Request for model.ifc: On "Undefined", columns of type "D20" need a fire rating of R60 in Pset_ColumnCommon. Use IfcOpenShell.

First a look at what the model holds.

```python
import ifcopenshell
import ifcopenshell.util.element

model = ifcopenshell.open("model.ifc")
print(model.schema)
storey = next(s for s in model.by_type("IfcBuildingStorey") if s.Name == "Undefined")
columns = [e for e in ifcopenshell.util.element.get_decomposition(storey) if e.is_a("IfcColumn")]
seen = {}
for e in columns:
    element_type = ifcopenshell.util.element.get_type(e)
    key = (element_type.Name if element_type != e and element_type else None, ifcopenshell.util.element.get_pset(e, "Pset_ColumnCommon", "FireRating"))
    seen[key] = seen.get(key, 0) + 1
for (name, value), count in sorted(seen.items(), key=str):
    print(count, "x", name, "|", value)
```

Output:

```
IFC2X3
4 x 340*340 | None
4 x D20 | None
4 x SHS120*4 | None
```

```python
import ifcopenshell
import ifcopenshell.api.pset
import ifcopenshell.util.element

model = ifcopenshell.open("model.ifc")

storey = next(s for s in model.by_type("IfcBuildingStorey") if s.Name == "Undefined")
columns = [e for e in ifcopenshell.util.element.get_decomposition(storey) if e.is_a("IfcColumn")]

count = 0
for e in columns:
    element_type = ifcopenshell.util.element.get_type(e)
    if element_type in (None, e) or element_type.Name != "D20":
        continue
    # add_pset returns the element's existing set when there is one.
    pset = ifcopenshell.api.pset.add_pset(model, product=e, name="Pset_ColumnCommon")
    ifcopenshell.api.pset.edit_pset(model, pset=pset, properties={"FireRating": "R60"})
    count += 1

print(count, "columns updated")

model.write("model-out.ifc")
```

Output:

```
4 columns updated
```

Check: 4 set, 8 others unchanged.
